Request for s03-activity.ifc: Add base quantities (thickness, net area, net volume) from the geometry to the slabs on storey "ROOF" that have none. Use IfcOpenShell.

First a look at what the model holds.

```python
import ifcopenshell
import ifcopenshell.util.element
import ifcopenshell.util.unit

model = ifcopenshell.open("s03-activity.ifc")
print(model.schema)
for unit_type in ("LENGTHUNIT", "AREAUNIT", "VOLUMEUNIT"):
    print(unit_type, ifcopenshell.util.unit.calculate_unit_scale(model, unit_type))
storey = next(s for s in model.by_type("IfcBuildingStorey") if s.Name == "ROOF")
slabs = [e for e in ifcopenshell.util.element.get_decomposition(storey) if e.is_a("IfcSlab")]
for e in sorted(slabs, key=lambda e: e.id()):
    print(e.id(), e.is_a(), e.Name, list(ifcopenshell.util.element.get_psets(e, qtos_only=True)), sep=" | ")
```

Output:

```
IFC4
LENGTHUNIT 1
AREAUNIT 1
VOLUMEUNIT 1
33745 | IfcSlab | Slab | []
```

```python
import ifcopenshell
import ifcopenshell.api.pset
import ifcopenshell.geom
import ifcopenshell.util.element
import ifcopenshell.util.shape
import ifcopenshell.util.unit

model = ifcopenshell.open("s03-activity.ifc")
unit_scale = ifcopenshell.util.unit.calculate_unit_scale(model)
area_scale = ifcopenshell.util.unit.calculate_unit_scale(model, "AREAUNIT")
volume_scale = ifcopenshell.util.unit.calculate_unit_scale(model, "VOLUMEUNIT")
settings = ifcopenshell.geom.settings()

storey = next(s for s in model.by_type("IfcBuildingStorey") if s.Name == "ROOF")
slabs = [e for e in ifcopenshell.util.element.get_decomposition(storey) if e.is_a("IfcSlab")]

for e in sorted(slabs, key=lambda e: e.id()):
    if ifcopenshell.util.element.get_psets(e, qtos_only=True, should_inherit=False):
        continue
    # Geometry comes back in metres, in the element's own axes.
    shape = ifcopenshell.geom.create_shape(settings, e)
    values = {
        "Width": ifcopenshell.util.shape.get_z(shape.geometry) / unit_scale,
        "NetArea": ifcopenshell.util.shape.get_footprint_area(shape.geometry) / area_scale,
        "NetVolume": ifcopenshell.util.shape.get_volume(shape.geometry) / volume_scale,
    }
    qto = ifcopenshell.api.pset.add_qto(model, product=e, name="Qto_SlabBaseQuantities")
    ifcopenshell.api.pset.edit_qto(model, qto=qto, properties=values)
    print(e.id(), {k: round(v, 3) for k, v in values.items()})

model.write("s03-activity-out.ifc")
```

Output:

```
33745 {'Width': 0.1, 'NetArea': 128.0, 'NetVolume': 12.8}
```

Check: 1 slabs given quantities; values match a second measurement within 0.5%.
